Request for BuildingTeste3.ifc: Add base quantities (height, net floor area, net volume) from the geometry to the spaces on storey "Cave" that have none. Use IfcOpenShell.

First a look at what the model holds.

```python
import ifcopenshell
import ifcopenshell.util.element
import ifcopenshell.util.unit

model = ifcopenshell.open("BuildingTeste3.ifc")
print(model.schema)
for unit_type in ("LENGTHUNIT", "AREAUNIT", "VOLUMEUNIT"):
    print(unit_type, ifcopenshell.util.unit.calculate_unit_scale(model, unit_type))
storey = next(s for s in model.by_type("IfcBuildingStorey") if s.Name == "Cave")
spaces = [e for e in ifcopenshell.util.element.get_decomposition(storey) if e.is_a("IfcSpace")]
for e in sorted(spaces, key=lambda e: e.id()):
    print(e.id(), e.is_a(), e.Name, list(ifcopenshell.util.element.get_psets(e, qtos_only=True)), sep=" | ")
```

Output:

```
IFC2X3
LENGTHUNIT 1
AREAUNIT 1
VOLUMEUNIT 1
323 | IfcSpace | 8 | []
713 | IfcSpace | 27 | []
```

```python
import ifcopenshell
import ifcopenshell.api.pset
import ifcopenshell.geom
import ifcopenshell.util.element
import ifcopenshell.util.shape
import ifcopenshell.util.unit

model = ifcopenshell.open("BuildingTeste3.ifc")
unit_scale = ifcopenshell.util.unit.calculate_unit_scale(model)
area_scale = ifcopenshell.util.unit.calculate_unit_scale(model, "AREAUNIT")
volume_scale = ifcopenshell.util.unit.calculate_unit_scale(model, "VOLUMEUNIT")
settings = ifcopenshell.geom.settings()

storey = next(s for s in model.by_type("IfcBuildingStorey") if s.Name == "Cave")
spaces = [e for e in ifcopenshell.util.element.get_decomposition(storey) if e.is_a("IfcSpace")]

for e in sorted(spaces, key=lambda e: e.id()):
    if ifcopenshell.util.element.get_psets(e, qtos_only=True, should_inherit=False):
        continue
    # Geometry comes back in metres, in the element's own axes.
    shape = ifcopenshell.geom.create_shape(settings, e)
    values = {
        "Height": ifcopenshell.util.shape.get_z(shape.geometry) / unit_scale,
        "NetFloorArea": ifcopenshell.util.shape.get_footprint_area(shape.geometry) / area_scale,
        "NetVolume": ifcopenshell.util.shape.get_volume(shape.geometry) / volume_scale,
    }
    qto = ifcopenshell.api.pset.add_qto(model, product=e, name="BaseQuantities")
    ifcopenshell.api.pset.edit_qto(model, qto=qto, properties=values)
    print(e.id(), {k: round(v, 3) for k, v in values.items()})

model.write("BuildingTeste3_edited.ifc")
```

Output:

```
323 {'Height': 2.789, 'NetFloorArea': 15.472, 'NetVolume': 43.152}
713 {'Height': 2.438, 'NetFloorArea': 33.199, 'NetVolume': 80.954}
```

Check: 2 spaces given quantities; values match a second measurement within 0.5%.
